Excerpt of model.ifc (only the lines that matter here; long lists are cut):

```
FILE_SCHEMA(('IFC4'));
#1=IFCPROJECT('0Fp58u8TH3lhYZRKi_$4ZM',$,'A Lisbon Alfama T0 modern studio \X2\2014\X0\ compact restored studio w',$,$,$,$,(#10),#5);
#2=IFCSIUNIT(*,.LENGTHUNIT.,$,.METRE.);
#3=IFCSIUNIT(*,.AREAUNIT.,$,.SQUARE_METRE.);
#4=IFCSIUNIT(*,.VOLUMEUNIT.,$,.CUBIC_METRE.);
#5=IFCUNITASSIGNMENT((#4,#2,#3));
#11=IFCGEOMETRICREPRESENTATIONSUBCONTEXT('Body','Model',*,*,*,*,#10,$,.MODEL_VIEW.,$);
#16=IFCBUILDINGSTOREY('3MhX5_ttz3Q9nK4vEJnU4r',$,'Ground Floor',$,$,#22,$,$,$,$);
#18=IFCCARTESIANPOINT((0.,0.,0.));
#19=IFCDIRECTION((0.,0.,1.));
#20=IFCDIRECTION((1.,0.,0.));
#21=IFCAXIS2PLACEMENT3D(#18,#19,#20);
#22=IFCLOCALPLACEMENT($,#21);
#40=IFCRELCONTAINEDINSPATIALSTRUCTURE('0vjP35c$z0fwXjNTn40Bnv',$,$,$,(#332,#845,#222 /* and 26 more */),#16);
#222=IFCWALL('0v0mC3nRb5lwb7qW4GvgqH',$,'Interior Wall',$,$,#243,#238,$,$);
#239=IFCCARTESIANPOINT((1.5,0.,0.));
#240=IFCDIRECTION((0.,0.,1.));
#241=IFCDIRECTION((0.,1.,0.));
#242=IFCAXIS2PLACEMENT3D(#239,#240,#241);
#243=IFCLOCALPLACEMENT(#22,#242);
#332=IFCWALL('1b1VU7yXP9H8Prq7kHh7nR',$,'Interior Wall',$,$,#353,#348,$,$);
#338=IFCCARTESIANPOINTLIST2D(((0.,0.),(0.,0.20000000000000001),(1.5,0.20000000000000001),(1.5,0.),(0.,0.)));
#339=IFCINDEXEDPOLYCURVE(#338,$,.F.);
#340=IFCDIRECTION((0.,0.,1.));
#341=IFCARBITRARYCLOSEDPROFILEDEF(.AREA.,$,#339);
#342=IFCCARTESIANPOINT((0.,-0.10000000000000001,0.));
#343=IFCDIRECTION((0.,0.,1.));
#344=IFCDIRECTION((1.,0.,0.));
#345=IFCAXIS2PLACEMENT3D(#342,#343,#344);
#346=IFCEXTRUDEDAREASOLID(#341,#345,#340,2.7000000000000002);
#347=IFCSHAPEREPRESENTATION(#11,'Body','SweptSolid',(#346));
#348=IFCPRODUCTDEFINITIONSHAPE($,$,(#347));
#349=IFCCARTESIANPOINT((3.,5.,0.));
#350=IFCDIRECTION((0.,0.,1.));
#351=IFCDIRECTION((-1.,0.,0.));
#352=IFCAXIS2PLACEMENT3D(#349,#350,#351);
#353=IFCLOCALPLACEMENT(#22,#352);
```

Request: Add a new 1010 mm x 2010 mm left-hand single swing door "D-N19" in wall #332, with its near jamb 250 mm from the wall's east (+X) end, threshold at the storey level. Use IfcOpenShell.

```python
import numpy as np
import ifcopenshell
import ifcopenshell.api.feature
import ifcopenshell.api.geometry
import ifcopenshell.api.root
import ifcopenshell.api.spatial
import ifcopenshell.geom
import ifcopenshell.util.element
import ifcopenshell.util.placement
import ifcopenshell.util.representation
import ifcopenshell.util.shape
import ifcopenshell.util.unit

model = ifcopenshell.open("model.ifc")
unit_scale = ifcopenshell.util.unit.calculate_unit_scale(model)
settings = ifcopenshell.geom.settings()


def volume(element):
    """Net volume in cubic metres, openings subtracted."""
    shape = ifcopenshell.geom.create_shape(settings, element)
    return ifcopenshell.util.shape.get_volume(shape.geometry)


wall = model.by_guid("1b1VU7yXP9H8Prq7kHh7nR")
storey = ifcopenshell.util.element.get_container(wall, ifc_class="IfcBuildingStorey")
context = ifcopenshell.util.representation.get_context(model, "Model", "Body", "MODEL_VIEW")
before = volume(wall)

width, height, from_end, sill = 1.01, 2.01, 0.25, 0.0  # metres

# The wall runs along its own X axis, and the end named is its -X end.
wall_shape = ifcopenshell.geom.create_shape(settings, wall)
x, y, z = ifcopenshell.util.shape.get_vertices(wall_shape.geometry).T
start = x.min() + from_end
face, thickness = float(y.min()), float(y.max() - y.min())
wall_matrix = ifcopenshell.util.placement.get_local_placement(wall.ObjectPlacement)
level = ifcopenshell.util.placement.get_local_placement(storey.ObjectPlacement)[2, 3]


def in_wall(x, y):
    """Placement at x, y metres in the wall's axes, at sill height."""
    matrix = wall_matrix.copy()
    matrix[:, 3] = wall_matrix @ np.array([x / unit_scale, y / unit_scale, 0.0, 1.0])
    matrix[2, 3] = level + sill / unit_scale
    return matrix


# Opening: a box that overshoots both wall faces by 50 mm.
opening = ifcopenshell.api.root.create_entity(model, ifc_class="IfcOpeningElement", predefined_type="OPENING")
box = ifcopenshell.api.geometry.add_wall_representation(
    model, context=context, length=width, height=height, thickness=thickness + 0.1
)
ifcopenshell.api.geometry.assign_representation(model, product=opening, representation=box)
ifcopenshell.api.geometry.edit_object_placement(model, product=opening, matrix=in_wall(start, face - 0.05), is_si=False)
ifcopenshell.api.feature.add_feature(model, feature=opening, element=wall)

door = ifcopenshell.api.root.create_entity(model, ifc_class="IfcDoor", name="D-N19", predefined_type="DOOR")
door.OverallWidth, door.OverallHeight = width / unit_scale, height / unit_scale
door.OperationType = "SINGLE_SWING_LEFT"
body = ifcopenshell.api.geometry.add_door_representation(
    model,
    context=context,
    overall_width=door.OverallWidth,
    overall_height=door.OverallHeight,
    operation_type="SINGLE_SWING_LEFT",
    lining_properties={"LiningDepth": thickness / unit_scale, "ThresholdDepth": thickness / unit_scale},
)
ifcopenshell.api.geometry.assign_representation(model, product=door, representation=body)
ifcopenshell.api.spatial.assign_container(model, products=[door], relating_structure=storey)
ifcopenshell.api.feature.add_filling(model, opening=opening, element=door)

# The lining spans the wall, so the door starts at the wall face.
ifcopenshell.api.geometry.edit_object_placement(model, product=door, matrix=in_wall(start, face), is_si=False)

after = volume(wall)

print(f"wall volume {before:.3f} -> {after:.3f} m3")

model.write("model_edited.ifc")
```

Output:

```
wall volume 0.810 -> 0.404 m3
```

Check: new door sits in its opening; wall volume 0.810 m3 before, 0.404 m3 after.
